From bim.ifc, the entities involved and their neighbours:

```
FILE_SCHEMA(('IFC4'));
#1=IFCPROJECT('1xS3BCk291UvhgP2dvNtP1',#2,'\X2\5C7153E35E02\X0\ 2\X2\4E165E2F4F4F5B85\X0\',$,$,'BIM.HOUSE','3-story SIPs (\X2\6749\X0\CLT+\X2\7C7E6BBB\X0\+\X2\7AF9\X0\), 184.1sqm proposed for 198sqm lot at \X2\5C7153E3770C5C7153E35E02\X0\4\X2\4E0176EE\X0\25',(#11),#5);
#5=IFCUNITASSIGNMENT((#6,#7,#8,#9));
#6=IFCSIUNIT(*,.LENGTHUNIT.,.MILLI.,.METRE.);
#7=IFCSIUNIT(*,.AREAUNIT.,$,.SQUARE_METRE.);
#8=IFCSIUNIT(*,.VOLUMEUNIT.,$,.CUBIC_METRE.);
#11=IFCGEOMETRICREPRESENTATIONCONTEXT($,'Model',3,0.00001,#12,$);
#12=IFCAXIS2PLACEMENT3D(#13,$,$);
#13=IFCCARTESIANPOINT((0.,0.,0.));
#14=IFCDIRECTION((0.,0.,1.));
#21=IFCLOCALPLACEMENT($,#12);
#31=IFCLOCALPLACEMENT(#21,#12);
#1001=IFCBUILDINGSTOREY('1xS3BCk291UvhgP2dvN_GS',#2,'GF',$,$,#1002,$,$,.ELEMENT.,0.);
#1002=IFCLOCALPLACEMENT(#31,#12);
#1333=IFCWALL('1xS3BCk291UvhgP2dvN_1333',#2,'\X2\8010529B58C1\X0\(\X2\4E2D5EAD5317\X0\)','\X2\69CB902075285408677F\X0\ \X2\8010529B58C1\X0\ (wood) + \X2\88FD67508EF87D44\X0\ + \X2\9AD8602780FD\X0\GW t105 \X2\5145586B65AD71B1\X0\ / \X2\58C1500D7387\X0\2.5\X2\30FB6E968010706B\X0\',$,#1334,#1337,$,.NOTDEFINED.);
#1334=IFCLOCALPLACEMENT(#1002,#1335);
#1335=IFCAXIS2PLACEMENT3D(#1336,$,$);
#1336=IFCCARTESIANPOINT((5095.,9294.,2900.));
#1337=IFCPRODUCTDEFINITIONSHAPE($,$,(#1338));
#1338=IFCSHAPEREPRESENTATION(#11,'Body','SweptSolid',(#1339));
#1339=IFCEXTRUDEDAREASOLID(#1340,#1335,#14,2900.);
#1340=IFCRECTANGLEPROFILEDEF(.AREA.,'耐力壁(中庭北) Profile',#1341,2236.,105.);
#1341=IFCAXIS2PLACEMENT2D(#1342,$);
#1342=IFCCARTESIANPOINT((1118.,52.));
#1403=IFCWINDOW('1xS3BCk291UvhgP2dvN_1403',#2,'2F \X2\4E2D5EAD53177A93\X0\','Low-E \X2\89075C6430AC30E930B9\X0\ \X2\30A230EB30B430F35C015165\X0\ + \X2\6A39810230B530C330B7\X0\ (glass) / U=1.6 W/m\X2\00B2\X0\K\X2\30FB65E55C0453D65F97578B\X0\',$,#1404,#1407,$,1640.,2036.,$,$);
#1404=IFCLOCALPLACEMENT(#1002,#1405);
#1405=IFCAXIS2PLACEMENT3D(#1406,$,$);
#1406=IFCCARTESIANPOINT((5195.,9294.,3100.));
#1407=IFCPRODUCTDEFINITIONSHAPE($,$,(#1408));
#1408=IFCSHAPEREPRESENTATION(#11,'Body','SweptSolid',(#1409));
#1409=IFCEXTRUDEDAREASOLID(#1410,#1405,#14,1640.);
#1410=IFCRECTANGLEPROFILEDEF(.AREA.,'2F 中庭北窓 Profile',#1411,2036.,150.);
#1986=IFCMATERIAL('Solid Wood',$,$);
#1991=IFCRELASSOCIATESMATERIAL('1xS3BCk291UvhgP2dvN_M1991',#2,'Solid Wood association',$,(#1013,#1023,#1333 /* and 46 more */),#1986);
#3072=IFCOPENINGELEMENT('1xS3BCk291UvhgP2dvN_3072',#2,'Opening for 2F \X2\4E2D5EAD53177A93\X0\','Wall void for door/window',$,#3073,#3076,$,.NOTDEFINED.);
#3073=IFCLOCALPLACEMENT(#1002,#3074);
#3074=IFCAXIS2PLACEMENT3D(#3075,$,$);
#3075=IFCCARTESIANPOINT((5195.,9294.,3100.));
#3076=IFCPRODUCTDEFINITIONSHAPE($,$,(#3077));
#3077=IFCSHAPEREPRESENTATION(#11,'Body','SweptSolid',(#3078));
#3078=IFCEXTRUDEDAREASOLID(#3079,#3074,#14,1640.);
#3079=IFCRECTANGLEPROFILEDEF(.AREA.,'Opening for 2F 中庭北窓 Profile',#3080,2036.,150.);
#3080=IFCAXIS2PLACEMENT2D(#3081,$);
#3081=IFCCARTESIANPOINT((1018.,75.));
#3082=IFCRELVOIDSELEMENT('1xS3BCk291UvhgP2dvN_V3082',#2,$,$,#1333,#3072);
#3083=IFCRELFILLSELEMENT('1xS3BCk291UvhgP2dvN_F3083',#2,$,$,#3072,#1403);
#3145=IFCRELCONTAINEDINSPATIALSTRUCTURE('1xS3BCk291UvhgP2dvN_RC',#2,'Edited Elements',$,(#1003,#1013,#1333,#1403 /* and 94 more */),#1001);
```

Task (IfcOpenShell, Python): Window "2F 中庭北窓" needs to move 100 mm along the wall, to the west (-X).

```python
import ifcopenshell
import ifcopenshell.api.geometry
import ifcopenshell.util.placement
import ifcopenshell.util.unit

model = ifcopenshell.open("bim.ifc")
unit_scale = ifcopenshell.util.unit.calculate_unit_scale(model)

window = model.by_guid("1xS3BCk291UvhgP2dvN_1403")
opening = window.FillsVoids[0].RelatingOpeningElement
wall = opening.VoidsElements[0].RelatingBuildingElement

wall_matrix = ifcopenshell.util.placement.get_local_placement(wall.ObjectPlacement)
shift = wall_matrix[:3, 0] * -0.1 / unit_scale
before = ifcopenshell.util.placement.get_local_placement(window.ObjectPlacement)[:3, 3].copy()

# The window is not placed relative to its opening, so move both.
for product in (opening, window):
    matrix = ifcopenshell.util.placement.get_local_placement(product.ObjectPlacement)
    matrix[:3, 3] += shift
    ifcopenshell.api.geometry.edit_object_placement(model, product=product, matrix=matrix, is_si=False)

after = ifcopenshell.util.placement.get_local_placement(window.ObjectPlacement)[:3, 3]
print("window moved by", (after - before).round(3) + 0.0)

model.write("bim-out.ifc")
```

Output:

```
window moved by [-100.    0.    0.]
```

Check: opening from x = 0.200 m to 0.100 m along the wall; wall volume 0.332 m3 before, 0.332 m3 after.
